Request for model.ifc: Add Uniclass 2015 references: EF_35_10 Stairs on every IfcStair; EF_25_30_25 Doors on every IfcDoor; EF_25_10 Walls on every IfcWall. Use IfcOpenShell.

First a look at what the model holds.

```python
import ifcopenshell

model = ifcopenshell.open("model.ifc")
print(model.schema)
print("classifications:", [c.Name for c in model.by_type("IfcClassification")])
for ifc_class in ("IfcDoor", "IfcRoof", "IfcStair", "IfcWall", "IfcWindow"):
    print(ifc_class, len(model.by_type(ifc_class)))
```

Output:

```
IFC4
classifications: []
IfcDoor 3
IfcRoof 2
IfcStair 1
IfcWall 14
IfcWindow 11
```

```python
import ifcopenshell
import ifcopenshell.api.classification

model = ifcopenshell.open("model.ifc")

system = ifcopenshell.api.classification.add_classification(model, classification="Uniclass 2015")

codes = {
    "IfcStair": ("EF_35_10", "Stairs"),
    "IfcDoor": ("EF_25_30_25", "Doors"),
    "IfcWall": ("EF_25_10", "Walls"),
}
for ifc_class, (code, name) in codes.items():
    products = model.by_type(ifc_class)
    ifcopenshell.api.classification.add_reference(
        model, products=products, classification=system, identification=code, name=name
    )
    print(code, len(products))

model.write("model_edited.ifc")
```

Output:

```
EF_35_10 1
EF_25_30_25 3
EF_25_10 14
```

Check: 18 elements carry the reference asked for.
